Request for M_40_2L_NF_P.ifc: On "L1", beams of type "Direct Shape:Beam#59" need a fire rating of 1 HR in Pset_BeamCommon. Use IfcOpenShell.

First a look at what the model holds.

```python
import ifcopenshell
import ifcopenshell.util.element

model = ifcopenshell.open("M_40_2L_NF_P.ifc")
print(model.schema)
storey = next(s for s in model.by_type("IfcBuildingStorey") if s.Name == "L1")
beams = [e for e in ifcopenshell.util.element.get_decomposition(storey) if e.is_a("IfcBeam")]
seen = {}
for e in beams:
    element_type = ifcopenshell.util.element.get_type(e)
    key = (element_type.Name if element_type != e and element_type else None, ifcopenshell.util.element.get_pset(e, "Pset_BeamCommon", "FireRating"))
    seen[key] = seen.get(key, 0) + 1
for (name, value), count in sorted(seen.items(), key=str):
    print(count, "x", name, "|", value)
```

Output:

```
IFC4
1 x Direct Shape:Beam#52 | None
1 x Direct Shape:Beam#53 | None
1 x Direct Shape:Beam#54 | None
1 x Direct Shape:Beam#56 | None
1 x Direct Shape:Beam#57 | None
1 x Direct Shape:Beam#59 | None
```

```python
import ifcopenshell
import ifcopenshell.api.pset
import ifcopenshell.util.element

model = ifcopenshell.open("M_40_2L_NF_P.ifc")

storey = next(s for s in model.by_type("IfcBuildingStorey") if s.Name == "L1")
beams = [e for e in ifcopenshell.util.element.get_decomposition(storey) if e.is_a("IfcBeam")]

count = 0
for e in beams:
    element_type = ifcopenshell.util.element.get_type(e)
    if element_type in (None, e) or element_type.Name != "Direct Shape:Beam#59":
        continue
    # add_pset returns the element's existing set when there is one.
    pset = ifcopenshell.api.pset.add_pset(model, product=e, name="Pset_BeamCommon")
    ifcopenshell.api.pset.edit_pset(model, pset=pset, properties={"FireRating": "1 HR"})
    count += 1

print(count, "beams updated")

model.write("M_40_2L_NF_P_updated.ifc")
```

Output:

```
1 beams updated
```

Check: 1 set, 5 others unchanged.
